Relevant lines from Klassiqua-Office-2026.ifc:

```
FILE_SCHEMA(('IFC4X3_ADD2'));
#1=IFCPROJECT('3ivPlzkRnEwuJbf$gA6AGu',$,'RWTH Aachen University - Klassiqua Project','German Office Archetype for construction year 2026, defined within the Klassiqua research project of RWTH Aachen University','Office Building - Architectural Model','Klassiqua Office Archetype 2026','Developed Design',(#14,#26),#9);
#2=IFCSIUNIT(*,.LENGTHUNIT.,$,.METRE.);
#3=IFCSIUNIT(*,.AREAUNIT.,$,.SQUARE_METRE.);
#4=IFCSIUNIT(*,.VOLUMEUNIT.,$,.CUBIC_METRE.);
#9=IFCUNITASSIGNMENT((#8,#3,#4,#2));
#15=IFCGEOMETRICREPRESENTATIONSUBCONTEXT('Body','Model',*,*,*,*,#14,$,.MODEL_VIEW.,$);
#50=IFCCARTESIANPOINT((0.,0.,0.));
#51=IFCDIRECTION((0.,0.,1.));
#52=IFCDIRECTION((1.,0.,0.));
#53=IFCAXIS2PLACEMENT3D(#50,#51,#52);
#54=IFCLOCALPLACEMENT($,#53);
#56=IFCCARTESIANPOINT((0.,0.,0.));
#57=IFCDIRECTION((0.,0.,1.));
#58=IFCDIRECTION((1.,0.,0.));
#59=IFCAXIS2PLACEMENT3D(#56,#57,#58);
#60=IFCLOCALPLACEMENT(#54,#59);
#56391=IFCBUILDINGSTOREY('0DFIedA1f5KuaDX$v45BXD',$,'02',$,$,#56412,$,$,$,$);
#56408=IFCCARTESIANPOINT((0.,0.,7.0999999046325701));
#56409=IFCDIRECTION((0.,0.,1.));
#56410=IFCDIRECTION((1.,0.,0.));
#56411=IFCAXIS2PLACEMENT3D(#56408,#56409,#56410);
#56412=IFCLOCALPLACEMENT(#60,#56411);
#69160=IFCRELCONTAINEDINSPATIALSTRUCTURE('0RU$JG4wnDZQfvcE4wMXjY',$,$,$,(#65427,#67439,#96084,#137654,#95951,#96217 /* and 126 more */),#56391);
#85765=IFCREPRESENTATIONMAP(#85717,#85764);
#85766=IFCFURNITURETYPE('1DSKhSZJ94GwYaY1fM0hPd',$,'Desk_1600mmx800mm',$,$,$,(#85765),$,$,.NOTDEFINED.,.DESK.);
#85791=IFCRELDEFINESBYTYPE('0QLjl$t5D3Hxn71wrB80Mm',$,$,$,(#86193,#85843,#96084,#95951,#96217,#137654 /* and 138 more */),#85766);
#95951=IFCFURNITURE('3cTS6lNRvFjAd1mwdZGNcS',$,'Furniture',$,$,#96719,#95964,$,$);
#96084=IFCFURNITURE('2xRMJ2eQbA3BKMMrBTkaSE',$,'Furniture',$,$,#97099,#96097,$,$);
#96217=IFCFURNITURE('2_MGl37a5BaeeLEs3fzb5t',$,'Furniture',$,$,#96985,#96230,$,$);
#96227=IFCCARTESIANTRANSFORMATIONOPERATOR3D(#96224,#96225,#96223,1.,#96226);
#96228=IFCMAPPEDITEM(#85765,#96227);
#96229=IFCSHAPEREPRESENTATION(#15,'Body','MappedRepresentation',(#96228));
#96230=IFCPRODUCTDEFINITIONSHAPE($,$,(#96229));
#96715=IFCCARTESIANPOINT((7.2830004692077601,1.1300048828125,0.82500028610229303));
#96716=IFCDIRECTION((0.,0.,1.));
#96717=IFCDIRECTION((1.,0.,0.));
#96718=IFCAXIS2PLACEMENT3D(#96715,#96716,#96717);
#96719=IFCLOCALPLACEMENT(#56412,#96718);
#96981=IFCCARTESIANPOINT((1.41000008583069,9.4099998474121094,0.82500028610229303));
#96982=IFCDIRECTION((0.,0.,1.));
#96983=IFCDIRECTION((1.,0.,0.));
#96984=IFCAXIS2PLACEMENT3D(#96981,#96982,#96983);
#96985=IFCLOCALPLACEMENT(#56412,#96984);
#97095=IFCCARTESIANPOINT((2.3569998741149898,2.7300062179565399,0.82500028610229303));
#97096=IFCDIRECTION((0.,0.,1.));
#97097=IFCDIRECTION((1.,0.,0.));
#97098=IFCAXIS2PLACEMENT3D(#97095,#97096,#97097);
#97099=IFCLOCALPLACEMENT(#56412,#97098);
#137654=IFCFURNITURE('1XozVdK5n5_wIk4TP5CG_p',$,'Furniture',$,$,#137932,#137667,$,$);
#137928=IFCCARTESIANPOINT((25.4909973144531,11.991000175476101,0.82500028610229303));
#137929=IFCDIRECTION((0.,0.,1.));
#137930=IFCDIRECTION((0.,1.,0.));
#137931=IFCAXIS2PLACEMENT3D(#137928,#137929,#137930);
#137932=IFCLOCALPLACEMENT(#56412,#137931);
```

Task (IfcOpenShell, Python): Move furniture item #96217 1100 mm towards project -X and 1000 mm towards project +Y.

```python
import ifcopenshell
import ifcopenshell.api.geometry
import ifcopenshell.util.placement

model = ifcopenshell.open("Klassiqua-Office-2026.ifc")

item = model.by_guid("2_MGl37a5BaeeLEs3fzb5t")
matrix = ifcopenshell.util.placement.get_local_placement(item.ObjectPlacement)
matrix[0, 3] -= 1.1
matrix[1, 3] += 1.0
ifcopenshell.api.geometry.edit_object_placement(model, product=item, matrix=matrix, is_si=False)

print(ifcopenshell.util.placement.get_local_placement(item.ObjectPlacement).round(3) + 0.0)

model.write("Klassiqua-Office-2026-out.ifc")
```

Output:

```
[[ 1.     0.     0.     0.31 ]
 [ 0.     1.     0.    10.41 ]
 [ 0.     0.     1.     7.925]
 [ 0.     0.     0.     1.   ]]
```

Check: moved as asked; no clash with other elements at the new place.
